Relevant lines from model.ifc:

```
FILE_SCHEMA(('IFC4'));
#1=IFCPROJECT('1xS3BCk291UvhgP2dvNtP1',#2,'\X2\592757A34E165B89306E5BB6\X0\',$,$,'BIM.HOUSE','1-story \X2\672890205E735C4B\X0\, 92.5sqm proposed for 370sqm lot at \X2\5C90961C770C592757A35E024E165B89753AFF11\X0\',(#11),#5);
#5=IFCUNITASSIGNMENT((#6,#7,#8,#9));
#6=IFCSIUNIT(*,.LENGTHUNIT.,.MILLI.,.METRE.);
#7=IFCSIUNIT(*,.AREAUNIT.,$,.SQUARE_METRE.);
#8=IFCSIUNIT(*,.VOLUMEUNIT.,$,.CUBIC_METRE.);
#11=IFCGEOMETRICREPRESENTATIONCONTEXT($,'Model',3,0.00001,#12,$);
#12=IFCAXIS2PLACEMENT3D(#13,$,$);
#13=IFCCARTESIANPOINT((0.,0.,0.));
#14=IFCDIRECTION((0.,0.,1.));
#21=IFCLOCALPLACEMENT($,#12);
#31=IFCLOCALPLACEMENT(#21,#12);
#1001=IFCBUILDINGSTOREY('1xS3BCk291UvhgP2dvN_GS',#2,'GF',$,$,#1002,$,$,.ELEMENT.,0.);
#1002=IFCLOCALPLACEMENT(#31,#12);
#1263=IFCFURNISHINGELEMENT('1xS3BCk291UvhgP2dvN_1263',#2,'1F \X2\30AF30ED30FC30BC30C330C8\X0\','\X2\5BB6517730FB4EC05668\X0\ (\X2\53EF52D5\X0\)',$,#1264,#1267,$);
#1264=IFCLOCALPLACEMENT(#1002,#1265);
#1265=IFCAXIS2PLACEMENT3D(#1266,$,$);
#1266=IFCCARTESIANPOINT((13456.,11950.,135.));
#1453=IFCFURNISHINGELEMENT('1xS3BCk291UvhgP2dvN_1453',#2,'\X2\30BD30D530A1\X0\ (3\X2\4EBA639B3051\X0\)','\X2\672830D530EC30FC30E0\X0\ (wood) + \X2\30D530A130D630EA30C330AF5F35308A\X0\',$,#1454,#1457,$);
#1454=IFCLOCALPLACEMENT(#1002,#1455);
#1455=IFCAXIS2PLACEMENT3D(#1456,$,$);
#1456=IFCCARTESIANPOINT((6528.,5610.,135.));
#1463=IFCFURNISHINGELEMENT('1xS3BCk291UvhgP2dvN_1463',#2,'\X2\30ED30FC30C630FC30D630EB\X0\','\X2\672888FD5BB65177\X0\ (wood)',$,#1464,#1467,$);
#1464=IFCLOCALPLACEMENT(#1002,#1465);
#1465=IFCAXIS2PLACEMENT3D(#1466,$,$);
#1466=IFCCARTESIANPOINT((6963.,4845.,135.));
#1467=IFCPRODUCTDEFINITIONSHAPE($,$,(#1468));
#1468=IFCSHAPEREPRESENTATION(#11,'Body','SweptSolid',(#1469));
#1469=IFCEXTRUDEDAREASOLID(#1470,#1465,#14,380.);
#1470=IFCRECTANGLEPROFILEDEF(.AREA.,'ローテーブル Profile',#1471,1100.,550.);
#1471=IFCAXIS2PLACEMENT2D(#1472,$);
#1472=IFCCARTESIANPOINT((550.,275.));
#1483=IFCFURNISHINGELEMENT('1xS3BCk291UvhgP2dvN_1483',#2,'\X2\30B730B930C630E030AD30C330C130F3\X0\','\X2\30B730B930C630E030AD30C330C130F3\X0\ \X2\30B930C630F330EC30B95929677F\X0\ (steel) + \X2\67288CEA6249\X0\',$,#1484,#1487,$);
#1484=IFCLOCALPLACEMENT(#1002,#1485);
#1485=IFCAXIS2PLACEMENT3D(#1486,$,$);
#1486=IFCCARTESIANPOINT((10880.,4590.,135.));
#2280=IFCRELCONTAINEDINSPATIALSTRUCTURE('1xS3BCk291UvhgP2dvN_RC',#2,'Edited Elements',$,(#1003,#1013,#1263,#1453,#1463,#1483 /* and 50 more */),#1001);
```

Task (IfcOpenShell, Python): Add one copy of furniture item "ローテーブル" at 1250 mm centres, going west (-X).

```python
import numpy as np
import ifcopenshell
import ifcopenshell.api.geometry
import ifcopenshell.api.root
import ifcopenshell.util.element
import ifcopenshell.util.placement
import ifcopenshell.util.unit

model = ifcopenshell.open("model.ifc")
unit_scale = ifcopenshell.util.unit.calculate_unit_scale(model)


def reuse_history(source, copy):
    """copy_class also copies each property set's owner history, people and application; keep the originals."""
    for rel in copy.IsDefinedBy:
        if rel.is_a("IfcRelDefinesByProperties") and (history := rel.RelatingPropertyDefinition.OwnerHistory):
            rel.RelatingPropertyDefinition.OwnerHistory = source.OwnerHistory
            ifcopenshell.util.element.remove_deep2(model, history)


source = model.by_guid("1xS3BCk291UvhgP2dvN_1463")
base = ifcopenshell.util.placement.get_local_placement(source.ObjectPlacement)
step = np.array([-1.0, 0.0, 0.0]) * 1.25 / unit_scale

for i in range(1, 2):
    copy = ifcopenshell.api.root.copy_class(model, product=source)
    copy.Representation = ifcopenshell.util.element.copy_deep(
        model, source.Representation, exclude=["IfcGeometricRepresentationContext", "IfcRepresentationMap"]
    )
    reuse_history(source, copy)
    matrix = base.copy()
    matrix[:3, 3] += i * step
    print("added at", matrix[:3, 3].round(3) + 0.0)
    ifcopenshell.api.geometry.edit_object_placement(model, product=copy, matrix=matrix, is_si=False)

model.write("model_edited.ifc")
```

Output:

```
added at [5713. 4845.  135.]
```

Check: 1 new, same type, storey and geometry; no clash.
